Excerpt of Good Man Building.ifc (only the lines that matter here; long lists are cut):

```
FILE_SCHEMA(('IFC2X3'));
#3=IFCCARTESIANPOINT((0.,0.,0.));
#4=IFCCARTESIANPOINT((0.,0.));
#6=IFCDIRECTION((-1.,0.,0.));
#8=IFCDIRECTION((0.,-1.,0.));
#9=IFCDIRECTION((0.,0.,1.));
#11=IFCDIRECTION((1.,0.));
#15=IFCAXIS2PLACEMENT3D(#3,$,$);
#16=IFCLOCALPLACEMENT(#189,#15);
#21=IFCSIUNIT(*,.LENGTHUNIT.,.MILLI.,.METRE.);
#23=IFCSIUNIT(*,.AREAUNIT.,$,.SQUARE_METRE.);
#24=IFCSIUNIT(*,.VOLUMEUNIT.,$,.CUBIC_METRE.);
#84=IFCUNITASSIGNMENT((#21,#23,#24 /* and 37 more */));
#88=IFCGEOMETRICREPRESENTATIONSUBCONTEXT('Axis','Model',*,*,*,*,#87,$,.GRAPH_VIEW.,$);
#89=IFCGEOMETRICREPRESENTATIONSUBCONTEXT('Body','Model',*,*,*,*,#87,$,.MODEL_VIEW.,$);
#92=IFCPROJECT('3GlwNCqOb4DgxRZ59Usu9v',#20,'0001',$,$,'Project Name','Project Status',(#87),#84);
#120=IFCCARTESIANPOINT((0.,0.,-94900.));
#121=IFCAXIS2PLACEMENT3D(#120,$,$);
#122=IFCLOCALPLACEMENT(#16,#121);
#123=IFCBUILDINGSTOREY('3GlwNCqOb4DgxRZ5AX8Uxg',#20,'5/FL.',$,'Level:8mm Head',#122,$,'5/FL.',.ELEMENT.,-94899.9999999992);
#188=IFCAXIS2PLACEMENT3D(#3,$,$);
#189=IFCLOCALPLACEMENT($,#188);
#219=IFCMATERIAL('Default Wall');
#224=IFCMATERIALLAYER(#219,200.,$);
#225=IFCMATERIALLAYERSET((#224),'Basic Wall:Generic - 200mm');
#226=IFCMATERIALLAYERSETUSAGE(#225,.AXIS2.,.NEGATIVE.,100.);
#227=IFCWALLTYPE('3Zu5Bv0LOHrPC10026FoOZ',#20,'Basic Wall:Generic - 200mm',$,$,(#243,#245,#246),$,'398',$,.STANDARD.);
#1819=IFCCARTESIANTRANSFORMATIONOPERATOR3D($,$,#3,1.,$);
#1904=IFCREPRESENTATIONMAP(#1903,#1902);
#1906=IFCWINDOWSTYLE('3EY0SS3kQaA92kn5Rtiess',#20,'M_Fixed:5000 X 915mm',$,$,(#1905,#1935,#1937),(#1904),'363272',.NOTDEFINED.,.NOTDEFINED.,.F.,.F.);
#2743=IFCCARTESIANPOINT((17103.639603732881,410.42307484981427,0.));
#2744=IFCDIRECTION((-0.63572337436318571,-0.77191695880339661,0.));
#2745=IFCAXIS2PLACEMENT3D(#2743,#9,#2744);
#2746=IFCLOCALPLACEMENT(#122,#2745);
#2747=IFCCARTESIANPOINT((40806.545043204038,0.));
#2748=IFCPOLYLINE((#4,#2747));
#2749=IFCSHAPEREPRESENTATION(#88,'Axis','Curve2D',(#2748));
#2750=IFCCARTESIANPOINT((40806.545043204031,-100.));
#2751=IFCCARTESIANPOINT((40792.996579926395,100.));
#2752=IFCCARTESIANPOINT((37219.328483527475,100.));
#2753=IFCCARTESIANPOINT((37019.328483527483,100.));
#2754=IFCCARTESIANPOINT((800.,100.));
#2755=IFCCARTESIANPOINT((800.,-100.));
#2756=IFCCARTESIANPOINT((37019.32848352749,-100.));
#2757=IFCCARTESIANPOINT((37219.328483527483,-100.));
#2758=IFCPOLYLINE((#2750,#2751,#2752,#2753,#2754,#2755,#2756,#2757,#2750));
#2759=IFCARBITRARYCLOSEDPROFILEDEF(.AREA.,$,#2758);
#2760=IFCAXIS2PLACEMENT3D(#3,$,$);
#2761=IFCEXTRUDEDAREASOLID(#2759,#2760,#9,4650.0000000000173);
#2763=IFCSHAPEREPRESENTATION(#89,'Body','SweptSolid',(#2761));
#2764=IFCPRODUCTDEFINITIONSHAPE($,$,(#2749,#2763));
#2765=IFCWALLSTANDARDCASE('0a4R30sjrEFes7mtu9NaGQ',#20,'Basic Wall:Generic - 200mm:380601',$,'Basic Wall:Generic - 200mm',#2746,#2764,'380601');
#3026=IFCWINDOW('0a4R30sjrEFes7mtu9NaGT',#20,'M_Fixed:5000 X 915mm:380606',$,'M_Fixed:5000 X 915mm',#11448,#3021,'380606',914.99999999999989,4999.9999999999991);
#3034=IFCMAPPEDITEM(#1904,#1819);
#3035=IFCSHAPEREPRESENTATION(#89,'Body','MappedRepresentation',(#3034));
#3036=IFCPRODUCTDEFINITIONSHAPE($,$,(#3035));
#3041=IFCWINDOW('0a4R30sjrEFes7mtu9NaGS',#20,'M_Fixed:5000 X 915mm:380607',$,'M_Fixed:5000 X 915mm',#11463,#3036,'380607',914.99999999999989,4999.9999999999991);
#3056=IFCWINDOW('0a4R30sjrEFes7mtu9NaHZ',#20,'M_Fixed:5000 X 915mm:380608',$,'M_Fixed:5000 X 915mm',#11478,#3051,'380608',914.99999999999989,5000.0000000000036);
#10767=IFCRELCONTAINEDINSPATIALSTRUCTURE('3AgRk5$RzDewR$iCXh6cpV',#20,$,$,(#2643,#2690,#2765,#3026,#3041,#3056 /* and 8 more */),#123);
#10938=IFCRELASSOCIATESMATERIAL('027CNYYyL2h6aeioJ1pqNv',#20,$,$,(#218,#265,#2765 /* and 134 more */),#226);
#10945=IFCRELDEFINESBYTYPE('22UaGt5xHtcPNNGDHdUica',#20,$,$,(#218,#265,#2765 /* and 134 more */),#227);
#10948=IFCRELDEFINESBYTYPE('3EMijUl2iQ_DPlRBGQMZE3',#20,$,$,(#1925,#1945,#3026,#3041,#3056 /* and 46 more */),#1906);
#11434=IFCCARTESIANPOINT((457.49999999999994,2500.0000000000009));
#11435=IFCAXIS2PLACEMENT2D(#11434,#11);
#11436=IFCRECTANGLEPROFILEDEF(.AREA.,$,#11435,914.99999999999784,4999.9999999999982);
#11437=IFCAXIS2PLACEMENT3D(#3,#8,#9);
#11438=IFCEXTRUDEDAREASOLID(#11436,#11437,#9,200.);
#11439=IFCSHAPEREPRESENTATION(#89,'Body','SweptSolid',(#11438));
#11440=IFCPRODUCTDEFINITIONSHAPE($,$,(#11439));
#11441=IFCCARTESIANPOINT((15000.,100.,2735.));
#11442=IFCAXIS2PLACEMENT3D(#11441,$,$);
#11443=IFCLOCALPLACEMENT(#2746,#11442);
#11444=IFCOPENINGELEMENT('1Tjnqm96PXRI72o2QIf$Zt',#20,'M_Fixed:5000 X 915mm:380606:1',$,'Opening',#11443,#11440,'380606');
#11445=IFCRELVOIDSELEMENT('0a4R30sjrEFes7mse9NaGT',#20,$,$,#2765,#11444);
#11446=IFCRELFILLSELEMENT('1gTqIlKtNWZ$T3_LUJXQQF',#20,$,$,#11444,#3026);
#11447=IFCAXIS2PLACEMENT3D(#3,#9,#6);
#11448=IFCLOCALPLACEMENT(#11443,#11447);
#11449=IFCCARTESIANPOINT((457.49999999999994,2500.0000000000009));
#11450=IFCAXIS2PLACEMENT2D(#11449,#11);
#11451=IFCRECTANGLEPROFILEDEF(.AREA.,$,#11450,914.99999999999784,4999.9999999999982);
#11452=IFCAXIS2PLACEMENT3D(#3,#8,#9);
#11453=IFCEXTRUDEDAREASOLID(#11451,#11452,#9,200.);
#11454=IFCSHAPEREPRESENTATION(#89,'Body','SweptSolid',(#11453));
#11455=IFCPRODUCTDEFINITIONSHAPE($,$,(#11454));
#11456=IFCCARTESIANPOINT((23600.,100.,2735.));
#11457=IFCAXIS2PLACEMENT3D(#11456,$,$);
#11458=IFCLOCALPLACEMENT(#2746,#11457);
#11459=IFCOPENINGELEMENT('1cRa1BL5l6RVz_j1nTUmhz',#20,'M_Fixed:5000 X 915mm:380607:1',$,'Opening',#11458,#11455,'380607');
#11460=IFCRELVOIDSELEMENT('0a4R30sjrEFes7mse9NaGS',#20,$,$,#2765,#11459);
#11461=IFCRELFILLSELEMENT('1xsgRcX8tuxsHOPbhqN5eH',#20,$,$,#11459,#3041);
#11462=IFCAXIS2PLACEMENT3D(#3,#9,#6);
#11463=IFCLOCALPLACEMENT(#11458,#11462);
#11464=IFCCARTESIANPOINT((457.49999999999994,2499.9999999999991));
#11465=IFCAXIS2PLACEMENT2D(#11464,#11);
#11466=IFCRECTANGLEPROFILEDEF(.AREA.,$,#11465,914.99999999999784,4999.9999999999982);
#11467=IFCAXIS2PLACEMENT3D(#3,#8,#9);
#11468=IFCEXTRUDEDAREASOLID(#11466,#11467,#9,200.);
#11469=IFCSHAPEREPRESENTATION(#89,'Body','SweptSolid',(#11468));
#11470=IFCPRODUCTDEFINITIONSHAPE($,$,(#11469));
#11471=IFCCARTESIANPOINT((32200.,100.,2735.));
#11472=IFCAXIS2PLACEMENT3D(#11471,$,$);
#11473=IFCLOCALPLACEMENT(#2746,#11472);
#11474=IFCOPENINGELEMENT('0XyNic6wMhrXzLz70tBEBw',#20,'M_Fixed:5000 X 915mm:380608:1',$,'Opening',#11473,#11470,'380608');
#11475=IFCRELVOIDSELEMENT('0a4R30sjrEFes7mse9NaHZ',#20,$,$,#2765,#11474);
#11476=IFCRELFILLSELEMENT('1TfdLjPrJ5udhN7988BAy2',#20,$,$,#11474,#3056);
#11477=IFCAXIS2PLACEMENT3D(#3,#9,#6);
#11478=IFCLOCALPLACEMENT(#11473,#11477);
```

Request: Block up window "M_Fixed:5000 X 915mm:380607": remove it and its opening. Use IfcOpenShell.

```python
import ifcopenshell
import ifcopenshell.api.feature
import ifcopenshell.api.root
import ifcopenshell.geom
import ifcopenshell.util.shape

model = ifcopenshell.open("Good Man Building.ifc")
settings = ifcopenshell.geom.settings()


def volume(element):
    """Net volume in cubic metres, openings subtracted."""
    shape = ifcopenshell.geom.create_shape(settings, element)
    return ifcopenshell.util.shape.get_volume(shape.geometry)


window = model.by_guid("0a4R30sjrEFes7mtu9NaGS")
opening = window.FillsVoids[0].RelatingOpeningElement
wall = opening.VoidsElements[0].RelatingBuildingElement
before = volume(wall)

ifcopenshell.api.root.remove_product(model, product=window)
ifcopenshell.api.feature.remove_feature(model, feature=opening)

after = volume(wall)

print(f"wall volume {before:.3f} -> {after:.3f} m3")

model.write("Good Man Building_rev.ifc")
```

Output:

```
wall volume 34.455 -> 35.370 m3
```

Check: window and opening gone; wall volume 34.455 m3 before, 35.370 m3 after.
